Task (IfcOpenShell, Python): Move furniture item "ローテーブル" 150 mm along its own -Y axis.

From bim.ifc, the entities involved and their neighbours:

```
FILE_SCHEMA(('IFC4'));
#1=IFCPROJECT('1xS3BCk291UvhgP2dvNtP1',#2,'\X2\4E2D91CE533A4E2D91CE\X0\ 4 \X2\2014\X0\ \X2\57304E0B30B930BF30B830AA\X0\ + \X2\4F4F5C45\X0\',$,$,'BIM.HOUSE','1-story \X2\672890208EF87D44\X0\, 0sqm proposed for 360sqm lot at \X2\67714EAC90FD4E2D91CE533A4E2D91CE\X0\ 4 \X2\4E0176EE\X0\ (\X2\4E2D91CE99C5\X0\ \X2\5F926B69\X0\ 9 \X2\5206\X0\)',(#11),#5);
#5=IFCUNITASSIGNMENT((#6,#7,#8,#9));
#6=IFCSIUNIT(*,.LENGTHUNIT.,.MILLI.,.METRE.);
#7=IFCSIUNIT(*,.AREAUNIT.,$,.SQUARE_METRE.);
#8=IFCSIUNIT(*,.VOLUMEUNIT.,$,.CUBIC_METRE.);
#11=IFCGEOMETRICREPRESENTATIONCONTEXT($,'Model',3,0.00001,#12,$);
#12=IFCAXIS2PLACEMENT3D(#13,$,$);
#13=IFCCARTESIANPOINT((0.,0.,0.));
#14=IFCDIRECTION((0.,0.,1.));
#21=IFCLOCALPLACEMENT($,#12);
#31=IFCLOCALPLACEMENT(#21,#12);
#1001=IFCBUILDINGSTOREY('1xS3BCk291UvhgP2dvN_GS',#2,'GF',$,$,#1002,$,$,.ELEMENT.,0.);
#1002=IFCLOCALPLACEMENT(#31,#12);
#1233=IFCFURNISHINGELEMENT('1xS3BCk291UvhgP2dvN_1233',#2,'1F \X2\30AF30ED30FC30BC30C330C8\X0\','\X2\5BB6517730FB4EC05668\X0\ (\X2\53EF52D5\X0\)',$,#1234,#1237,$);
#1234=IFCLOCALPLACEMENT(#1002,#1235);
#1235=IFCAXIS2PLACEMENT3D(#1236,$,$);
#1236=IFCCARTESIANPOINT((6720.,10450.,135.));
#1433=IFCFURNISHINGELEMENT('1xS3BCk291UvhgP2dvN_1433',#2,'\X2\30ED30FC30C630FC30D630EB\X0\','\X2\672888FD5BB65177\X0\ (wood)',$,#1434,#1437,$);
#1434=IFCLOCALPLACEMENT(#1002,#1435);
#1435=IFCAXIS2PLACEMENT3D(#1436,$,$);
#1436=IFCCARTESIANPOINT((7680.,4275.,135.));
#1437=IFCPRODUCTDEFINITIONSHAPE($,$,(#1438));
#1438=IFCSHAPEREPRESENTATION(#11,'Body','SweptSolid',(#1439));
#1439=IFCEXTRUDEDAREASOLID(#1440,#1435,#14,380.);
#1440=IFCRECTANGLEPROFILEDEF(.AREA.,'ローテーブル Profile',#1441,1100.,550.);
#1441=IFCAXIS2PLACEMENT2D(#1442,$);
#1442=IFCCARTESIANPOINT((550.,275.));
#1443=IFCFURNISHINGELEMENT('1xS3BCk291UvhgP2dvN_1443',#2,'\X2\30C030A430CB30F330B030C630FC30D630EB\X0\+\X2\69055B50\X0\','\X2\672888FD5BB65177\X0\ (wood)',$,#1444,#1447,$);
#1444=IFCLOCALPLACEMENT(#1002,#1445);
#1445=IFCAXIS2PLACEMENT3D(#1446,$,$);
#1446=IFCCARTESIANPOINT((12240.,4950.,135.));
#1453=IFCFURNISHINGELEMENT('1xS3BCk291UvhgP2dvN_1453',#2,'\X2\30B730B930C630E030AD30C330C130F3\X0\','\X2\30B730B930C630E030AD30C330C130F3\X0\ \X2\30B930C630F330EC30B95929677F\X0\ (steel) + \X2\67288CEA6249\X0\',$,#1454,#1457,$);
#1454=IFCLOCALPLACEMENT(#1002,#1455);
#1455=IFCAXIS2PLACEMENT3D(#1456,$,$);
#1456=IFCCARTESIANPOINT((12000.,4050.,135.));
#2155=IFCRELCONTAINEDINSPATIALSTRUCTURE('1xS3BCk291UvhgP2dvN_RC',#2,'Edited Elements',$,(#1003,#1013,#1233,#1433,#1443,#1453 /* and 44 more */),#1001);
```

```python
import ifcopenshell
import ifcopenshell.api.geometry
import ifcopenshell.util.placement
import ifcopenshell.util.unit

model = ifcopenshell.open("bim.ifc")
unit_scale = ifcopenshell.util.unit.calculate_unit_scale(model)

item = model.by_guid("1xS3BCk291UvhgP2dvN_1433")
matrix = ifcopenshell.util.placement.get_local_placement(item.ObjectPlacement)
matrix[:3, 3] -= matrix[:3, 1] * 0.15 / unit_scale
ifcopenshell.api.geometry.edit_object_placement(model, product=item, matrix=matrix, is_si=False)

print(ifcopenshell.util.placement.get_local_placement(item.ObjectPlacement).round(3) + 0.0)

model.write("bim-out.ifc")
```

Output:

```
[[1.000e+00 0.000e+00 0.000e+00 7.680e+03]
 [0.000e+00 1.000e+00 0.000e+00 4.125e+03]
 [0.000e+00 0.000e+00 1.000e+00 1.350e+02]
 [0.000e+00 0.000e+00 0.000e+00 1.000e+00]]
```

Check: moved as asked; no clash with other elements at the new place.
